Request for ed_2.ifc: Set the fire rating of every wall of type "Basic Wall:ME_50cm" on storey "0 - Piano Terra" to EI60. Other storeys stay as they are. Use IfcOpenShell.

First a look at what the model holds.

```python
import ifcopenshell
import ifcopenshell.util.element

model = ifcopenshell.open("ed_2.ifc")
print(model.schema)
storey = next(s for s in model.by_type("IfcBuildingStorey") if s.Name == "0 - Piano Terra")
walls = [e for e in ifcopenshell.util.element.get_decomposition(storey) if e.is_a("IfcWall")]
seen = {}
for e in walls:
    element_type = ifcopenshell.util.element.get_type(e)
    key = (element_type.Name if element_type != e and element_type else None, ifcopenshell.util.element.get_pset(e, "Pset_WallCommon", "FireRating"))
    seen[key] = seen.get(key, 0) + 1
for (name, value), count in sorted(seen.items(), key=str):
    print(count, "x", name, "|", value)
```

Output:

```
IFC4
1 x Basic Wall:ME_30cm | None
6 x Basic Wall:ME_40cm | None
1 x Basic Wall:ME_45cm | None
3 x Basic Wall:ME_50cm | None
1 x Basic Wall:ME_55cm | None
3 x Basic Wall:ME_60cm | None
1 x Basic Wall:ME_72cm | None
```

```python
import ifcopenshell
import ifcopenshell.api.pset
import ifcopenshell.util.element

model = ifcopenshell.open("ed_2.ifc")

storey = next(s for s in model.by_type("IfcBuildingStorey") if s.Name == "0 - Piano Terra")
walls = [e for e in ifcopenshell.util.element.get_decomposition(storey) if e.is_a("IfcWall")]

count = 0
for e in walls:
    element_type = ifcopenshell.util.element.get_type(e)
    if element_type in (None, e) or element_type.Name != "Basic Wall:ME_50cm":
        continue
    # add_pset returns the element's existing set when there is one.
    pset = ifcopenshell.api.pset.add_pset(model, product=e, name="Pset_WallCommon")
    ifcopenshell.api.pset.edit_pset(model, pset=pset, properties={"FireRating": "EI60"})
    count += 1

print(count, "walls updated")

model.write("ed_2_edited.ifc")
```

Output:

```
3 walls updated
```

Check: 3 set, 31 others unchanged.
